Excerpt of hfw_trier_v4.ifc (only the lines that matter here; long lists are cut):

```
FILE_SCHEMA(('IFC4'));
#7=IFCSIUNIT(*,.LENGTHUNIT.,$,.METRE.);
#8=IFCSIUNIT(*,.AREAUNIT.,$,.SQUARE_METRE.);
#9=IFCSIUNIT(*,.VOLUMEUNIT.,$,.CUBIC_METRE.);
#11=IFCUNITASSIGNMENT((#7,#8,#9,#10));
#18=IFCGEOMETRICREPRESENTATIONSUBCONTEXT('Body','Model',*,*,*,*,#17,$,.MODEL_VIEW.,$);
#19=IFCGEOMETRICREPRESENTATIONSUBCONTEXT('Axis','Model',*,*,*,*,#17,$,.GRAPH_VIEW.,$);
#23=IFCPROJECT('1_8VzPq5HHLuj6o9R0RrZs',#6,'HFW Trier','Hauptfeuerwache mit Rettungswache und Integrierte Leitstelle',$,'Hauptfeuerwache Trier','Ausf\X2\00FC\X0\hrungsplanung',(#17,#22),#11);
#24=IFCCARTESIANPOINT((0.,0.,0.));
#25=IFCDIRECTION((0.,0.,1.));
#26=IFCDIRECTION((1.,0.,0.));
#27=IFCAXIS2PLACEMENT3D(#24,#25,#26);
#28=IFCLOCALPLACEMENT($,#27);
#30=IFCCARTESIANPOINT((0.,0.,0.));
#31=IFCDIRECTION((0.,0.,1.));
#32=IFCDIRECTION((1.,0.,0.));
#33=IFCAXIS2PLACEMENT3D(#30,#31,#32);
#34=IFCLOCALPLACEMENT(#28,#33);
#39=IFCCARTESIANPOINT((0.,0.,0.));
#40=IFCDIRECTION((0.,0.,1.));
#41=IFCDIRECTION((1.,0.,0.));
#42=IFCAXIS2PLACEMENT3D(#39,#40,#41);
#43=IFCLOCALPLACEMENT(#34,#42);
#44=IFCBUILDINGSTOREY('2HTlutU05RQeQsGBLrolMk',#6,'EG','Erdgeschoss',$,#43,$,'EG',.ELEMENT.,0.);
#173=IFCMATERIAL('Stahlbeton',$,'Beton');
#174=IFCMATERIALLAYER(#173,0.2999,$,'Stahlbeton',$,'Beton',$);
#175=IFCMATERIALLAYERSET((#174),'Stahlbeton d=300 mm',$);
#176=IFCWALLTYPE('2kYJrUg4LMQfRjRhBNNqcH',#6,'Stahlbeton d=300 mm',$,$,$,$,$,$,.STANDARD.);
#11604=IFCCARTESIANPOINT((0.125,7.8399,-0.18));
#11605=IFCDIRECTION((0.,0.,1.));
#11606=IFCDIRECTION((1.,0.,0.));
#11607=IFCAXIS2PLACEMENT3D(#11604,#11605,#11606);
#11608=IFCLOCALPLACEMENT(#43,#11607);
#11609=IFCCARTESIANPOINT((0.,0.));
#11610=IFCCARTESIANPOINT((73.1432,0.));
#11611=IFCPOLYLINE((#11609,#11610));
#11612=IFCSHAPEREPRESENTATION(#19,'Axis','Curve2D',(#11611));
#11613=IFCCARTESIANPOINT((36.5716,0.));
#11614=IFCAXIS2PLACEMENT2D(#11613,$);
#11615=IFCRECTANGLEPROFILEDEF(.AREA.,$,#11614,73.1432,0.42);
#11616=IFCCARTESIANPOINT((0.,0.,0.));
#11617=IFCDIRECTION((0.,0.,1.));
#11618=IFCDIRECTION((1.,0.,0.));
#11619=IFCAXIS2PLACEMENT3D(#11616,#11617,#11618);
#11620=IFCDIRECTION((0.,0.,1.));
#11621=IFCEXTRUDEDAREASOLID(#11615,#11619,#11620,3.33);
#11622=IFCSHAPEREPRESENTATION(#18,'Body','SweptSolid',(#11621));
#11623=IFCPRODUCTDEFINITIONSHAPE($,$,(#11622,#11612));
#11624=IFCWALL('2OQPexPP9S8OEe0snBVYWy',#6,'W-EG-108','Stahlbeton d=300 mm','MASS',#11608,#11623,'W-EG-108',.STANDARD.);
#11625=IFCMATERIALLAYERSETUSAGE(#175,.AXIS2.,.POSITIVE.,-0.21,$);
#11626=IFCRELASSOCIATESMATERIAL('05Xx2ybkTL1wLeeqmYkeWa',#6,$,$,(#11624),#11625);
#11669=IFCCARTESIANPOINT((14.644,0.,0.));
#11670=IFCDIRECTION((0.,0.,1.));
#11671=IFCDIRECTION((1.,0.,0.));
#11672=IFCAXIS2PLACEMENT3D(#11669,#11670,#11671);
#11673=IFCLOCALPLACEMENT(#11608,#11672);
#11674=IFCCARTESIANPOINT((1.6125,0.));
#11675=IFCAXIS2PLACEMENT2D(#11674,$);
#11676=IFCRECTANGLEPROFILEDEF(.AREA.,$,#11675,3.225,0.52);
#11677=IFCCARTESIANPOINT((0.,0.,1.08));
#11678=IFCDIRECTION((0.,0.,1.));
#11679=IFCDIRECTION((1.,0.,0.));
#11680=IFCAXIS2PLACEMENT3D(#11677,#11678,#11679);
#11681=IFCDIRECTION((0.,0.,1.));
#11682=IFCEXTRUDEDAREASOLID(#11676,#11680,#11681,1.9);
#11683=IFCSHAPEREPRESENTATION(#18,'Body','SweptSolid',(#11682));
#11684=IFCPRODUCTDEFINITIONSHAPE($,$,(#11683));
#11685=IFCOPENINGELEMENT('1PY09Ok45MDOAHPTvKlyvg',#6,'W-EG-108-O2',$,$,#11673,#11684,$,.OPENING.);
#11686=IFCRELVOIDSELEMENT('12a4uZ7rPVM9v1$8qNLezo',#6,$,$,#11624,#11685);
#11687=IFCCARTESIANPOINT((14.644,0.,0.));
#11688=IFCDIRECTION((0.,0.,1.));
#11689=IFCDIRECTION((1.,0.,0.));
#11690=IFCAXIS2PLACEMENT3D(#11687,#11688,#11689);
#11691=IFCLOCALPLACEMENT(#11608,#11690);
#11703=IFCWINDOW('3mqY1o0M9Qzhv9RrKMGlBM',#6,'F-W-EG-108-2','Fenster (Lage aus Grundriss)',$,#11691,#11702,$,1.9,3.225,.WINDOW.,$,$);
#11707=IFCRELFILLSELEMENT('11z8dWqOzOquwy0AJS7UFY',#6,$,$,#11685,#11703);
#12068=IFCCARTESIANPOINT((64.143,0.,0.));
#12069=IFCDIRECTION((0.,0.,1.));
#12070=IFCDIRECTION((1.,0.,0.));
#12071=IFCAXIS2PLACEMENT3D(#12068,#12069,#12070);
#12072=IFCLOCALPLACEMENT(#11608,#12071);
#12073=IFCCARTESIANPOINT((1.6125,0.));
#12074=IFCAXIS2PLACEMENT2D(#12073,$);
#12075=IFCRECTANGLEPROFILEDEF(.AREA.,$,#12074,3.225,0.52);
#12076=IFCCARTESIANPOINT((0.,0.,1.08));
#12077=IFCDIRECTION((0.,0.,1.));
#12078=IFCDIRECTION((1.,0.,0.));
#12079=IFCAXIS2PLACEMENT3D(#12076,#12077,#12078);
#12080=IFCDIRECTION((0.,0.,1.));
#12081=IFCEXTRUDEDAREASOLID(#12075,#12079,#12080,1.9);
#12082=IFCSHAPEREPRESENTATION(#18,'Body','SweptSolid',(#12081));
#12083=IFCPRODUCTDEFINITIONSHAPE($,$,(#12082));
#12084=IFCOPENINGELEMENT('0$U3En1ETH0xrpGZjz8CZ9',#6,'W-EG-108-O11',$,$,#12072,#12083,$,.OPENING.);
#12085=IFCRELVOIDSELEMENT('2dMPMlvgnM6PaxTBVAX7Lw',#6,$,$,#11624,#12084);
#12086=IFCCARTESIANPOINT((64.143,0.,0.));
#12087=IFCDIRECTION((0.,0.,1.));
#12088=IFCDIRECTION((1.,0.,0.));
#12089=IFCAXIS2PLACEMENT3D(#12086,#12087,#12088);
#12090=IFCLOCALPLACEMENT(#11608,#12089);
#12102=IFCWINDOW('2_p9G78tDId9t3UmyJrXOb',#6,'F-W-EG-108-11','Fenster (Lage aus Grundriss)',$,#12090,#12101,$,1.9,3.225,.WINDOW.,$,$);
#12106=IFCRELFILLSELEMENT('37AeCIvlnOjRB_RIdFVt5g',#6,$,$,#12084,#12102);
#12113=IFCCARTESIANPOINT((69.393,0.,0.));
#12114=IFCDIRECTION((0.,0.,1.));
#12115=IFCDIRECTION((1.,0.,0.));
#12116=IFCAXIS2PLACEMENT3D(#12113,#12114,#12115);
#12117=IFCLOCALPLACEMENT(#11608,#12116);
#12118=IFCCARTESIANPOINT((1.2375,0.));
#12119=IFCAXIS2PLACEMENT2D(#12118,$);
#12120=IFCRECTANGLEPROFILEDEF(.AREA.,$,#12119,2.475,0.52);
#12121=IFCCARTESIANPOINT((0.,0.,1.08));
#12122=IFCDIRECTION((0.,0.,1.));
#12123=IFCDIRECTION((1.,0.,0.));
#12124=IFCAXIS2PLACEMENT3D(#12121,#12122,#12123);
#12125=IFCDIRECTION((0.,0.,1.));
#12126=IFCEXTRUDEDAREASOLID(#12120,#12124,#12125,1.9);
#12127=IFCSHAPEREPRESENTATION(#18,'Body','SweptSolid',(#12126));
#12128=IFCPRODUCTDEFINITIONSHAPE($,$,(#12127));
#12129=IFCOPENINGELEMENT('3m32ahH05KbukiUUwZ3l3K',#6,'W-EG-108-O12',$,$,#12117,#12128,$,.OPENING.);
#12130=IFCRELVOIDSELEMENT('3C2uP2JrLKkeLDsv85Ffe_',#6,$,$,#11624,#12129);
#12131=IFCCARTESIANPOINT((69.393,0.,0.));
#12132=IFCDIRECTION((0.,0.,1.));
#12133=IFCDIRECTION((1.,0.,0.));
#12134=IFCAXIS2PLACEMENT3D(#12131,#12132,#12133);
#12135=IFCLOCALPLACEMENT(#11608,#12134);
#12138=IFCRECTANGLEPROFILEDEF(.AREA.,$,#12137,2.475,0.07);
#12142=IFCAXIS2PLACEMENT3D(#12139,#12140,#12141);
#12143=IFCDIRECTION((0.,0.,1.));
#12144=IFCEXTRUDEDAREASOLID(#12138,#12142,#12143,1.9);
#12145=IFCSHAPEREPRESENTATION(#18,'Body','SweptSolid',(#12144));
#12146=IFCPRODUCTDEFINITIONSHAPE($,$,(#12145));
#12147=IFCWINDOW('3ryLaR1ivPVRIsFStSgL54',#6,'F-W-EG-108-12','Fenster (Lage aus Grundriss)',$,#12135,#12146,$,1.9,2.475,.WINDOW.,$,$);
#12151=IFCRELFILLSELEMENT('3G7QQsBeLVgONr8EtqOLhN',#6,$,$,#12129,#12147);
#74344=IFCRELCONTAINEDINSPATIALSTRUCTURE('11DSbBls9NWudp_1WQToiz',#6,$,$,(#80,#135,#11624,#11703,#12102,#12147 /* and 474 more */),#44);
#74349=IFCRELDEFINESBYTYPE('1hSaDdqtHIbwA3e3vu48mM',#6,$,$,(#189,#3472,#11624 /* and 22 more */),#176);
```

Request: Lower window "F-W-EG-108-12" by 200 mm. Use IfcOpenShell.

```python
import numpy as np
import ifcopenshell
import ifcopenshell.api.geometry
import ifcopenshell.util.placement
import ifcopenshell.util.unit

model = ifcopenshell.open("hfw_trier_v4.ifc")
unit_scale = ifcopenshell.util.unit.calculate_unit_scale(model)

window = model.by_guid("3ryLaR1ivPVRIsFStSgL54")
opening = window.FillsVoids[0].RelatingOpeningElement
dz = -0.2

shift = np.array([0.0, 0.0, dz])
# The window is not placed relative to its opening, so move both.
for product in (opening, window):
    matrix = ifcopenshell.util.placement.get_local_placement(product.ObjectPlacement)
    matrix[:3, 3] += shift
    ifcopenshell.api.geometry.edit_object_placement(model, product=product, matrix=matrix, is_si=False)

print(f"moved by {dz * unit_scale:+.3f} m")

model.write("hfw_trier_v4_v2.ifc")
```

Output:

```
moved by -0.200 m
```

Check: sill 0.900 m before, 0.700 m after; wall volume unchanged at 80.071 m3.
